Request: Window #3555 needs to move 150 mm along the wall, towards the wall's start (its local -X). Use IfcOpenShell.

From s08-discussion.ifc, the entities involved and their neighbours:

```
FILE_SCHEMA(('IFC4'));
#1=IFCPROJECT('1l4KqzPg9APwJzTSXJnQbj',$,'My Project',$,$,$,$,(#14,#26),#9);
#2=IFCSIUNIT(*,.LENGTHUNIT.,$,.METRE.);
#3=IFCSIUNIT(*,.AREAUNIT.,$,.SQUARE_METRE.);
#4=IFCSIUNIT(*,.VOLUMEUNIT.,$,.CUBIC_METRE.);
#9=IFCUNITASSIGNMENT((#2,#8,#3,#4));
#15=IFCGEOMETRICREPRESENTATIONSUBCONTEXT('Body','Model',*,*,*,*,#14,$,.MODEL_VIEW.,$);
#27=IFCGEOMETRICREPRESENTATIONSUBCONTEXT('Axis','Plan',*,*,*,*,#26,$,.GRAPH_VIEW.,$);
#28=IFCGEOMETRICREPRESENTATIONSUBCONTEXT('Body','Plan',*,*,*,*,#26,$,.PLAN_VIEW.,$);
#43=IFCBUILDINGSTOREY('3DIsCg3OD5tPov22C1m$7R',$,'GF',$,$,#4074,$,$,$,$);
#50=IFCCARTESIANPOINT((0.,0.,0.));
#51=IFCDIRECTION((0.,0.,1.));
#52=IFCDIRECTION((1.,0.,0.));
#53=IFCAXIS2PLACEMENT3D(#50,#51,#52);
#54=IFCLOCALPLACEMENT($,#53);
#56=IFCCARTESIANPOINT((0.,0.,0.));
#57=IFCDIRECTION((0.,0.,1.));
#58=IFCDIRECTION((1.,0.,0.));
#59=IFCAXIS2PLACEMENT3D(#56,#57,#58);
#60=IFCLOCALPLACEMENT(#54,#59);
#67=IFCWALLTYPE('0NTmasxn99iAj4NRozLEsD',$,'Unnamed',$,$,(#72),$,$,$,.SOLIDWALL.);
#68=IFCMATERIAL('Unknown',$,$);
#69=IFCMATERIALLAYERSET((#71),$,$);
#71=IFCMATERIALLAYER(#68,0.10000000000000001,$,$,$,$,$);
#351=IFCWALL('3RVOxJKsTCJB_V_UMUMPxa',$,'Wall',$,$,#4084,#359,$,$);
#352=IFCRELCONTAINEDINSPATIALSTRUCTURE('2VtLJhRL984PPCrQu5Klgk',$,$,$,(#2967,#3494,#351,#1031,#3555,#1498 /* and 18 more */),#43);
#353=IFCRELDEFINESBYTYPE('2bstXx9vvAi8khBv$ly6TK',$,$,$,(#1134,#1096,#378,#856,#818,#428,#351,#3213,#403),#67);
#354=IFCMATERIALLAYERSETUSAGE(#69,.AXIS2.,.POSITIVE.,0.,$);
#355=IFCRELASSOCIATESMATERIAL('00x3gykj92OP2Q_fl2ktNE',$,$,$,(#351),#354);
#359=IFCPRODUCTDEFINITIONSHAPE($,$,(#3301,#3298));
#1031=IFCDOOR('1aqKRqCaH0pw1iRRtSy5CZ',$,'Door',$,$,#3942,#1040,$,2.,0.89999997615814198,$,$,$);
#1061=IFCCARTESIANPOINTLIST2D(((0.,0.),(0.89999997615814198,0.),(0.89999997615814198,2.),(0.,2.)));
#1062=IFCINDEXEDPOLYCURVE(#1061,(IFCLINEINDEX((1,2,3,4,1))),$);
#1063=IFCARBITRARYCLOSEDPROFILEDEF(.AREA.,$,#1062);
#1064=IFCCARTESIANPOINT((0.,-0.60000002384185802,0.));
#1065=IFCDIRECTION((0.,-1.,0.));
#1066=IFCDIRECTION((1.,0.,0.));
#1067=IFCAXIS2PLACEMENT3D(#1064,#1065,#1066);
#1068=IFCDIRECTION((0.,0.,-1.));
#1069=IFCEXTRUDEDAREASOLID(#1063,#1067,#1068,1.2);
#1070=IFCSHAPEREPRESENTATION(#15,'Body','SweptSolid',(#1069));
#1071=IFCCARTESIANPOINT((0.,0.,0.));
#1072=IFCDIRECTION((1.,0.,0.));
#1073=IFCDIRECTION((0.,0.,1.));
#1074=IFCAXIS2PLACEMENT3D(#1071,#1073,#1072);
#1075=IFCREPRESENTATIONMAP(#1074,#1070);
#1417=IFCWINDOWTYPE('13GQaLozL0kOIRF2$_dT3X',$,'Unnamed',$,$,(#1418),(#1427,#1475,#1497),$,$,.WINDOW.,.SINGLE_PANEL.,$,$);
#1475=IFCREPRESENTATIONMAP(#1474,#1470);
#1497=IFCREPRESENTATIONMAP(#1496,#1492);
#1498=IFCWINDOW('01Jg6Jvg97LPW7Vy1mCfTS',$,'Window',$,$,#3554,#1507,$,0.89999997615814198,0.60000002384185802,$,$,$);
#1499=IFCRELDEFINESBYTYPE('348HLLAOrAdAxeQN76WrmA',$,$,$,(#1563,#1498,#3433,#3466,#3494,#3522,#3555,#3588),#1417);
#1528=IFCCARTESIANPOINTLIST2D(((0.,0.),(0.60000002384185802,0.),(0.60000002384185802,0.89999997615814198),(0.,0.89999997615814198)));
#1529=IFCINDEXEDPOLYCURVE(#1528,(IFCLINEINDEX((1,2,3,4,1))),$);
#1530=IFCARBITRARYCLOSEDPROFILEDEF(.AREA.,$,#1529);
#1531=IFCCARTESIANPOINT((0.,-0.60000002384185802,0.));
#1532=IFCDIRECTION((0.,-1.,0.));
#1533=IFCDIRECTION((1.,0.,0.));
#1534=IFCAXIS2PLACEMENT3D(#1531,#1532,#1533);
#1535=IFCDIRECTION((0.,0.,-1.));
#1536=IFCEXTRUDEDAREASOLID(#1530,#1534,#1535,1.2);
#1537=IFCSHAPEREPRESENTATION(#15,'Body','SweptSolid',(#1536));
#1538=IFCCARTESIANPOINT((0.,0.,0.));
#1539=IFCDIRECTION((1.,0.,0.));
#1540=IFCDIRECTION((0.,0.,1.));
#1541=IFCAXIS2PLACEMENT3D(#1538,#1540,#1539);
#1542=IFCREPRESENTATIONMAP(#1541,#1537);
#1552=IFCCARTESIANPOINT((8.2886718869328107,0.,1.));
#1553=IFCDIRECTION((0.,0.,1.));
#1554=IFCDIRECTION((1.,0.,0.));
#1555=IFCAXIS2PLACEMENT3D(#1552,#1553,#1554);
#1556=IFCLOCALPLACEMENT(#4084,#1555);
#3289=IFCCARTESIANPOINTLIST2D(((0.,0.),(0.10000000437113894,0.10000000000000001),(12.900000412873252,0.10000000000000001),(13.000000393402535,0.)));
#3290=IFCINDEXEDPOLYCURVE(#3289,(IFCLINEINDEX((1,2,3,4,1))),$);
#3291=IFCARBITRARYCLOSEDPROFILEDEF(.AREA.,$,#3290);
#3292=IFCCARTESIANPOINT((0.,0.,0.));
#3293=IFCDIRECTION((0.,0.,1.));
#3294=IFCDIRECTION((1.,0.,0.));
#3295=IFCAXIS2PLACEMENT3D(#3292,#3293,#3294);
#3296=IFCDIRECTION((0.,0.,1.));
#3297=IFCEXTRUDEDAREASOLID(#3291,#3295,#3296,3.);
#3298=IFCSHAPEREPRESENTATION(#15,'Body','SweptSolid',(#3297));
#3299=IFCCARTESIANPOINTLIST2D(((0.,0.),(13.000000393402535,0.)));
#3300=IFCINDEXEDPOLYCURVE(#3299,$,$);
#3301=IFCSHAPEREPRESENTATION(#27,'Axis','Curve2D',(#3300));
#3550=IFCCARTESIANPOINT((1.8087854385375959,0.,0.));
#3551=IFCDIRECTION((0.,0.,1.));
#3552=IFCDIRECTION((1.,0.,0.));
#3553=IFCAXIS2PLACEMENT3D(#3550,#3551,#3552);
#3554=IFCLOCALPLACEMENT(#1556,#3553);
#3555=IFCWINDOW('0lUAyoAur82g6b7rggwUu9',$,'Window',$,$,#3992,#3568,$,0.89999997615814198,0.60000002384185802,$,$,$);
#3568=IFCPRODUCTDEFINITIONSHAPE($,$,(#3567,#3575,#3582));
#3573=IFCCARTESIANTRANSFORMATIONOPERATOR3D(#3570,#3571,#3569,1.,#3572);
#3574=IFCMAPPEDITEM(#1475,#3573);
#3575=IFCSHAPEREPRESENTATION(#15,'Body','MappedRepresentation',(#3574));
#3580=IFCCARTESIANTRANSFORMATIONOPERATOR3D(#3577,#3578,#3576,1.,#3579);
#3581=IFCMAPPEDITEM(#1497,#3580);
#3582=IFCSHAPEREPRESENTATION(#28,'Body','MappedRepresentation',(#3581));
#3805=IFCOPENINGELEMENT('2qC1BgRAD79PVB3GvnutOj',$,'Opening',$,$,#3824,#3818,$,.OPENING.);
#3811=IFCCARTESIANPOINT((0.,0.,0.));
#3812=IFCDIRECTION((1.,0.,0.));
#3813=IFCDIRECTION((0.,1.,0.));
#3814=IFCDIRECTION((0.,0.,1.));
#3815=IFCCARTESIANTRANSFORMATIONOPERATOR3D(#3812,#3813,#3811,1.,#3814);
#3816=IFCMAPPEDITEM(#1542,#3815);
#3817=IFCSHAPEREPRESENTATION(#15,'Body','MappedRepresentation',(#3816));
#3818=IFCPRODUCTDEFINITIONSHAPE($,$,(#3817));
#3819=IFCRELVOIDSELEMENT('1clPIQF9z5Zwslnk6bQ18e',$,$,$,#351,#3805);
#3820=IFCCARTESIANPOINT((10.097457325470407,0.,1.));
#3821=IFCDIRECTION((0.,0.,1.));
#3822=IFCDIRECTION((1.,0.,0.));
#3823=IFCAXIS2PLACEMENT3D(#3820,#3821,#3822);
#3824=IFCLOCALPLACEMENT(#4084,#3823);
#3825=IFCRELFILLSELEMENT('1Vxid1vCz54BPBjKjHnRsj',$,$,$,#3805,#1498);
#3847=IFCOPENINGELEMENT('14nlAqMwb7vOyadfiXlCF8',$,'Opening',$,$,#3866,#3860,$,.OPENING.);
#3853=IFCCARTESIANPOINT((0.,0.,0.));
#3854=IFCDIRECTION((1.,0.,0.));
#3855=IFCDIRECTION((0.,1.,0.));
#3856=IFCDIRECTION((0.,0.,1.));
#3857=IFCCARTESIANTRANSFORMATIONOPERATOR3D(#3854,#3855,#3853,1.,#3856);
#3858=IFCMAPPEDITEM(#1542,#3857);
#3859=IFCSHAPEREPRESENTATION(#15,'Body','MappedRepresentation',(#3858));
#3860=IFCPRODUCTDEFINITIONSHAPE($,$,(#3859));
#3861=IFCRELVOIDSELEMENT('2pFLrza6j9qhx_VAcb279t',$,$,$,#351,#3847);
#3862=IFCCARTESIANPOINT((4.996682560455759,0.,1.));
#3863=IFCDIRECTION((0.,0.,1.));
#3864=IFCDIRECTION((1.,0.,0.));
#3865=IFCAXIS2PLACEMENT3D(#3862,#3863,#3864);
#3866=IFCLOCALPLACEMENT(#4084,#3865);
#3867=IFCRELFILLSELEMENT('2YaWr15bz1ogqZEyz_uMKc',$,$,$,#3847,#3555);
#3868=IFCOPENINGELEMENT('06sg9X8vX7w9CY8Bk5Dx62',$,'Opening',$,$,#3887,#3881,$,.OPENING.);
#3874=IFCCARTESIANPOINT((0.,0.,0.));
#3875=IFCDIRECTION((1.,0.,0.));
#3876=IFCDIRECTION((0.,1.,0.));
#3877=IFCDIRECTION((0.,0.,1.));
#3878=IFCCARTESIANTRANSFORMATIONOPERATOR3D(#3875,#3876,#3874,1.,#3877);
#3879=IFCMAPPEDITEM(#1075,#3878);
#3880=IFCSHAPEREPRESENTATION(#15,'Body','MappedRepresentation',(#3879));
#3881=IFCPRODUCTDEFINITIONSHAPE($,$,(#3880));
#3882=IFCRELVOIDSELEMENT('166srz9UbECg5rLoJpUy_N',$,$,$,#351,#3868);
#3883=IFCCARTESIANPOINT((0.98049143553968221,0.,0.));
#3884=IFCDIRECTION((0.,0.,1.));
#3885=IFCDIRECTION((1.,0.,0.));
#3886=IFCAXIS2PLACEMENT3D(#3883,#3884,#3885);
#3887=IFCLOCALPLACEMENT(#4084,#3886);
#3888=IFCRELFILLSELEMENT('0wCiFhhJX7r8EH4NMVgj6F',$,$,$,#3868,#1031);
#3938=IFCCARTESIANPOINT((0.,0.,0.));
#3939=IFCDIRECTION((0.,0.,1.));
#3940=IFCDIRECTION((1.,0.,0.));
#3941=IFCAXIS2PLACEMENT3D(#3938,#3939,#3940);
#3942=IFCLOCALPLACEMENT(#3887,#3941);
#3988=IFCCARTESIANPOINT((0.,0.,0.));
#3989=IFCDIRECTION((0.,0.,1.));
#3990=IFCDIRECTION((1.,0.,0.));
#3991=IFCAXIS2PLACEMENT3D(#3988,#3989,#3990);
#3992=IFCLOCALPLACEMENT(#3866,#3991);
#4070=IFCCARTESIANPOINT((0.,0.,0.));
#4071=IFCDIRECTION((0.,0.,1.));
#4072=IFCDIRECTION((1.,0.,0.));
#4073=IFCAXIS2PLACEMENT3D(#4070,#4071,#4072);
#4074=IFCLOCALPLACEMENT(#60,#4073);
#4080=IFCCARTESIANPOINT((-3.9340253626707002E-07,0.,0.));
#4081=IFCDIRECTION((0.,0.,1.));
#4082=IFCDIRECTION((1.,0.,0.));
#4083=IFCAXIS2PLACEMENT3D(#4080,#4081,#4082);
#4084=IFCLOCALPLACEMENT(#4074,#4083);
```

```python
import ifcopenshell
import ifcopenshell.api.geometry
import ifcopenshell.util.placement
import ifcopenshell.util.unit

model = ifcopenshell.open("s08-discussion.ifc")
unit_scale = ifcopenshell.util.unit.calculate_unit_scale(model)

window = model.by_guid("0lUAyoAur82g6b7rggwUu9")
opening = window.FillsVoids[0].RelatingOpeningElement
wall = opening.VoidsElements[0].RelatingBuildingElement

wall_matrix = ifcopenshell.util.placement.get_local_placement(wall.ObjectPlacement)
shift = wall_matrix[:3, 0] * -0.15 / unit_scale
before = ifcopenshell.util.placement.get_local_placement(window.ObjectPlacement)[:3, 3].copy()

# The window is placed relative to its opening, so it follows when the opening moves.
matrix = ifcopenshell.util.placement.get_local_placement(opening.ObjectPlacement)
matrix[:3, 3] += shift
ifcopenshell.api.geometry.edit_object_placement(
    model, product=opening, matrix=matrix, is_si=False, should_transform_children=True
)

after = ifcopenshell.util.placement.get_local_placement(window.ObjectPlacement)[:3, 3]
print("window moved by", (after - before).round(3) + 0.0)

model.write("s08-discussion_v2.ifc")
```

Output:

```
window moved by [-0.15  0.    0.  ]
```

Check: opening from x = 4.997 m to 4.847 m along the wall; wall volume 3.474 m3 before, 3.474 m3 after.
